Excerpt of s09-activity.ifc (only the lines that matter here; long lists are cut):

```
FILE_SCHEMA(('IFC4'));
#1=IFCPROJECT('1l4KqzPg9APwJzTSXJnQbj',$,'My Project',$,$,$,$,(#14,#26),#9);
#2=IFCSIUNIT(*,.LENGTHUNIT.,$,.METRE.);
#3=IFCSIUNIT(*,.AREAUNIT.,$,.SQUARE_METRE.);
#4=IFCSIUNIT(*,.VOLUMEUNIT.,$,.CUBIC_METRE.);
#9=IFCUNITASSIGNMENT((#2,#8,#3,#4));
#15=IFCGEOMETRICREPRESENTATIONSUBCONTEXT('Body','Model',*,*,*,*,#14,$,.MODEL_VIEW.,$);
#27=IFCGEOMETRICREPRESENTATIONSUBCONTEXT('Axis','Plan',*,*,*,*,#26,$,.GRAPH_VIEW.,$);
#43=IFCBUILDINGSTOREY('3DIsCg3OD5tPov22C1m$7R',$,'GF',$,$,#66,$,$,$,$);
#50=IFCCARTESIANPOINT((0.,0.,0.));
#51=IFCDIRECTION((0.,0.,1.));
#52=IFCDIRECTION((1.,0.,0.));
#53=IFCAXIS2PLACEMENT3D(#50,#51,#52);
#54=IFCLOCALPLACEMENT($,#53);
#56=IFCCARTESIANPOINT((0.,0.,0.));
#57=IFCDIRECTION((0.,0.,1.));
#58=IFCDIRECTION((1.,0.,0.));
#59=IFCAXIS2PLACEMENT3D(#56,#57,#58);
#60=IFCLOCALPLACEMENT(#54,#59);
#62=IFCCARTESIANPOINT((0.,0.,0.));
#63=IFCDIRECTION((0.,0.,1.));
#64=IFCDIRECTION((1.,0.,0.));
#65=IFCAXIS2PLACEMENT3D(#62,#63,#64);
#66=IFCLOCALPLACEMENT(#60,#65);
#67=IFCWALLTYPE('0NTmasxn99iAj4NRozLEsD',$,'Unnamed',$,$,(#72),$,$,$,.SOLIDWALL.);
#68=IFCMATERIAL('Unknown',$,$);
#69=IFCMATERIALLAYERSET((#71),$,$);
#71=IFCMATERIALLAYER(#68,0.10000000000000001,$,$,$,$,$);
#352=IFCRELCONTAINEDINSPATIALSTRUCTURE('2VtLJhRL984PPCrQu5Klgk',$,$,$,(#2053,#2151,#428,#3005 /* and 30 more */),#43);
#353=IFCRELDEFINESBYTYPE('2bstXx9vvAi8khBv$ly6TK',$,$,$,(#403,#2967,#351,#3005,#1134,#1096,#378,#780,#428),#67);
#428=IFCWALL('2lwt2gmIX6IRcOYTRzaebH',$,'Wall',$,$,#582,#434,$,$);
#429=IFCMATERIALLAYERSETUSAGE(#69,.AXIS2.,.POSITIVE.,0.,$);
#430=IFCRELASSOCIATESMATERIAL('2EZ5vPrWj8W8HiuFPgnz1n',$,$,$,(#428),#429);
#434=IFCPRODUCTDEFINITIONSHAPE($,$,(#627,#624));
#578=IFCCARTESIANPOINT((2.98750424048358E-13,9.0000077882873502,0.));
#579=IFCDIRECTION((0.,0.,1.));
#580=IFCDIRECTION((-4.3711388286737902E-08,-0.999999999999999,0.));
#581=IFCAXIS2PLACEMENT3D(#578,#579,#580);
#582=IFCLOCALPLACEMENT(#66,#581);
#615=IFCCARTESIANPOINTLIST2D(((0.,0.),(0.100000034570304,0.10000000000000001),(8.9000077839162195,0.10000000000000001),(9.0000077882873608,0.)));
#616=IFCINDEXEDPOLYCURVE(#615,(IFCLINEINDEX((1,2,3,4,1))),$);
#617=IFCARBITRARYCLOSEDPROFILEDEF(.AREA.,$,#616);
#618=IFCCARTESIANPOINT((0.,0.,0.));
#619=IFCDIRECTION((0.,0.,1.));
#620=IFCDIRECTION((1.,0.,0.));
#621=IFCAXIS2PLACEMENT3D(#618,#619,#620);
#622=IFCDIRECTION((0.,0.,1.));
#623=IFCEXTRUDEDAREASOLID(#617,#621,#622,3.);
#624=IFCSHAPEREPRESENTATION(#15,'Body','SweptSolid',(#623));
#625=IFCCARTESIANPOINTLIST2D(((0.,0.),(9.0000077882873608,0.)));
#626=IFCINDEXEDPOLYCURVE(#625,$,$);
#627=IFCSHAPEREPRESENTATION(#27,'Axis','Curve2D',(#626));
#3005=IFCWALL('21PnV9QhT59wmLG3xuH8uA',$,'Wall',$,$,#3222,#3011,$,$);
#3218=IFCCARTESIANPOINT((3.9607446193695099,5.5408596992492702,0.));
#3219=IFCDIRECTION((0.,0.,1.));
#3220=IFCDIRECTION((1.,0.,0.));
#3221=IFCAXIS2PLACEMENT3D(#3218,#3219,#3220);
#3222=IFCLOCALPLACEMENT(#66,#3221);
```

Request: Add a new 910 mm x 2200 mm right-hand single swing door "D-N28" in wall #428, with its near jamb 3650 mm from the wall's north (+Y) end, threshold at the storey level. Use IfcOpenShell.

```python
import numpy as np
import ifcopenshell
import ifcopenshell.api.feature
import ifcopenshell.api.geometry
import ifcopenshell.api.root
import ifcopenshell.api.spatial
import ifcopenshell.geom
import ifcopenshell.util.element
import ifcopenshell.util.placement
import ifcopenshell.util.representation
import ifcopenshell.util.shape
import ifcopenshell.util.unit

model = ifcopenshell.open("s09-activity.ifc")
unit_scale = ifcopenshell.util.unit.calculate_unit_scale(model)
settings = ifcopenshell.geom.settings()


def volume(element):
    """Net volume in cubic metres, openings subtracted."""
    shape = ifcopenshell.geom.create_shape(settings, element)
    return ifcopenshell.util.shape.get_volume(shape.geometry)


wall = model.by_guid("2lwt2gmIX6IRcOYTRzaebH")
storey = ifcopenshell.util.element.get_container(wall, ifc_class="IfcBuildingStorey")
context = ifcopenshell.util.representation.get_context(model, "Model", "Body", "MODEL_VIEW")
before = volume(wall)

width, height, from_end, sill = 0.91, 2.2, 3.65, 0.0  # metres

# The wall runs along its own X axis, and the end named is its -X end.
wall_shape = ifcopenshell.geom.create_shape(settings, wall)
x, y, z = ifcopenshell.util.shape.get_vertices(wall_shape.geometry).T
start = x.min() + from_end
face, thickness = float(y.min()), float(y.max() - y.min())
wall_matrix = ifcopenshell.util.placement.get_local_placement(wall.ObjectPlacement)
level = ifcopenshell.util.placement.get_local_placement(storey.ObjectPlacement)[2, 3]


def in_wall(x, y):
    """Placement at x, y metres in the wall's axes, at sill height."""
    matrix = wall_matrix.copy()
    matrix[:, 3] = wall_matrix @ np.array([x / unit_scale, y / unit_scale, 0.0, 1.0])
    matrix[2, 3] = level + sill / unit_scale
    return matrix


# Opening: a box that overshoots both wall faces by 50 mm.
opening = ifcopenshell.api.root.create_entity(model, ifc_class="IfcOpeningElement", predefined_type="OPENING")
box = ifcopenshell.api.geometry.add_wall_representation(
    model, context=context, length=width, height=height, thickness=thickness + 0.1
)
ifcopenshell.api.geometry.assign_representation(model, product=opening, representation=box)
ifcopenshell.api.geometry.edit_object_placement(model, product=opening, matrix=in_wall(start, face - 0.05), is_si=False)
ifcopenshell.api.feature.add_feature(model, feature=opening, element=wall)

door = ifcopenshell.api.root.create_entity(model, ifc_class="IfcDoor", name="D-N28", predefined_type="DOOR")
door.OverallWidth, door.OverallHeight = width / unit_scale, height / unit_scale
door.OperationType = "SINGLE_SWING_RIGHT"
body = ifcopenshell.api.geometry.add_door_representation(
    model,
    context=context,
    overall_width=door.OverallWidth,
    overall_height=door.OverallHeight,
    operation_type="SINGLE_SWING_RIGHT",
    lining_properties={"LiningDepth": thickness / unit_scale, "ThresholdDepth": thickness / unit_scale},
)
ifcopenshell.api.geometry.assign_representation(model, product=door, representation=body)
ifcopenshell.api.spatial.assign_container(model, products=[door], relating_structure=storey)
ifcopenshell.api.feature.add_filling(model, opening=opening, element=door)

# The lining spans the wall, so the door starts at the wall face.
ifcopenshell.api.geometry.edit_object_placement(model, product=door, matrix=in_wall(start, face), is_si=False)

after = volume(wall)

print(f"wall volume {before:.3f} -> {after:.3f} m3")

model.write("s09-activity_rev.ifc")
```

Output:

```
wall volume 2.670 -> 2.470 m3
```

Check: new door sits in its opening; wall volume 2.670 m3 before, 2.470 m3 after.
